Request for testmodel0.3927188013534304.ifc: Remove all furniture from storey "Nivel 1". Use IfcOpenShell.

First a look at what the model holds.

```python
import ifcopenshell
import ifcopenshell.util.element

model = ifcopenshell.open("testmodel0.3927188013534304.ifc")
print(model.schema)
storey = next(s for s in model.by_type("IfcBuildingStorey") if s.Name == "Nivel 1")
furniture = [e for e in ifcopenshell.util.element.get_decomposition(storey) if e.is_a("IfcFurnishingElement")]
seen = {}
for e in furniture:
    element_type = ifcopenshell.util.element.get_type(e)
    name = element_type.Name if element_type not in (None, e) else None
    seen[name] = seen.get(name, 0) + 1
for name, count in sorted(seen.items(), key=str):
    print(count, "x", name)
```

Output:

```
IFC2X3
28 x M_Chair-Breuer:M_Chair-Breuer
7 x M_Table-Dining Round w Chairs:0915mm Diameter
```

```python
import ifcopenshell
import ifcopenshell.api.root
import ifcopenshell.util.element

model = ifcopenshell.open("testmodel0.3927188013534304.ifc")

storey = next(s for s in model.by_type("IfcBuildingStorey") if s.Name == "Nivel 1")
furniture = [e for e in ifcopenshell.util.element.get_decomposition(storey) if e.is_a("IfcFurnishingElement")]

for e in furniture:
    ifcopenshell.api.root.remove_product(model, product=e)
print(len(furniture), "removed")

model.write("testmodel0.3927188013534304_v2.ifc")
```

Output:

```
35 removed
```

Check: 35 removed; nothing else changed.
